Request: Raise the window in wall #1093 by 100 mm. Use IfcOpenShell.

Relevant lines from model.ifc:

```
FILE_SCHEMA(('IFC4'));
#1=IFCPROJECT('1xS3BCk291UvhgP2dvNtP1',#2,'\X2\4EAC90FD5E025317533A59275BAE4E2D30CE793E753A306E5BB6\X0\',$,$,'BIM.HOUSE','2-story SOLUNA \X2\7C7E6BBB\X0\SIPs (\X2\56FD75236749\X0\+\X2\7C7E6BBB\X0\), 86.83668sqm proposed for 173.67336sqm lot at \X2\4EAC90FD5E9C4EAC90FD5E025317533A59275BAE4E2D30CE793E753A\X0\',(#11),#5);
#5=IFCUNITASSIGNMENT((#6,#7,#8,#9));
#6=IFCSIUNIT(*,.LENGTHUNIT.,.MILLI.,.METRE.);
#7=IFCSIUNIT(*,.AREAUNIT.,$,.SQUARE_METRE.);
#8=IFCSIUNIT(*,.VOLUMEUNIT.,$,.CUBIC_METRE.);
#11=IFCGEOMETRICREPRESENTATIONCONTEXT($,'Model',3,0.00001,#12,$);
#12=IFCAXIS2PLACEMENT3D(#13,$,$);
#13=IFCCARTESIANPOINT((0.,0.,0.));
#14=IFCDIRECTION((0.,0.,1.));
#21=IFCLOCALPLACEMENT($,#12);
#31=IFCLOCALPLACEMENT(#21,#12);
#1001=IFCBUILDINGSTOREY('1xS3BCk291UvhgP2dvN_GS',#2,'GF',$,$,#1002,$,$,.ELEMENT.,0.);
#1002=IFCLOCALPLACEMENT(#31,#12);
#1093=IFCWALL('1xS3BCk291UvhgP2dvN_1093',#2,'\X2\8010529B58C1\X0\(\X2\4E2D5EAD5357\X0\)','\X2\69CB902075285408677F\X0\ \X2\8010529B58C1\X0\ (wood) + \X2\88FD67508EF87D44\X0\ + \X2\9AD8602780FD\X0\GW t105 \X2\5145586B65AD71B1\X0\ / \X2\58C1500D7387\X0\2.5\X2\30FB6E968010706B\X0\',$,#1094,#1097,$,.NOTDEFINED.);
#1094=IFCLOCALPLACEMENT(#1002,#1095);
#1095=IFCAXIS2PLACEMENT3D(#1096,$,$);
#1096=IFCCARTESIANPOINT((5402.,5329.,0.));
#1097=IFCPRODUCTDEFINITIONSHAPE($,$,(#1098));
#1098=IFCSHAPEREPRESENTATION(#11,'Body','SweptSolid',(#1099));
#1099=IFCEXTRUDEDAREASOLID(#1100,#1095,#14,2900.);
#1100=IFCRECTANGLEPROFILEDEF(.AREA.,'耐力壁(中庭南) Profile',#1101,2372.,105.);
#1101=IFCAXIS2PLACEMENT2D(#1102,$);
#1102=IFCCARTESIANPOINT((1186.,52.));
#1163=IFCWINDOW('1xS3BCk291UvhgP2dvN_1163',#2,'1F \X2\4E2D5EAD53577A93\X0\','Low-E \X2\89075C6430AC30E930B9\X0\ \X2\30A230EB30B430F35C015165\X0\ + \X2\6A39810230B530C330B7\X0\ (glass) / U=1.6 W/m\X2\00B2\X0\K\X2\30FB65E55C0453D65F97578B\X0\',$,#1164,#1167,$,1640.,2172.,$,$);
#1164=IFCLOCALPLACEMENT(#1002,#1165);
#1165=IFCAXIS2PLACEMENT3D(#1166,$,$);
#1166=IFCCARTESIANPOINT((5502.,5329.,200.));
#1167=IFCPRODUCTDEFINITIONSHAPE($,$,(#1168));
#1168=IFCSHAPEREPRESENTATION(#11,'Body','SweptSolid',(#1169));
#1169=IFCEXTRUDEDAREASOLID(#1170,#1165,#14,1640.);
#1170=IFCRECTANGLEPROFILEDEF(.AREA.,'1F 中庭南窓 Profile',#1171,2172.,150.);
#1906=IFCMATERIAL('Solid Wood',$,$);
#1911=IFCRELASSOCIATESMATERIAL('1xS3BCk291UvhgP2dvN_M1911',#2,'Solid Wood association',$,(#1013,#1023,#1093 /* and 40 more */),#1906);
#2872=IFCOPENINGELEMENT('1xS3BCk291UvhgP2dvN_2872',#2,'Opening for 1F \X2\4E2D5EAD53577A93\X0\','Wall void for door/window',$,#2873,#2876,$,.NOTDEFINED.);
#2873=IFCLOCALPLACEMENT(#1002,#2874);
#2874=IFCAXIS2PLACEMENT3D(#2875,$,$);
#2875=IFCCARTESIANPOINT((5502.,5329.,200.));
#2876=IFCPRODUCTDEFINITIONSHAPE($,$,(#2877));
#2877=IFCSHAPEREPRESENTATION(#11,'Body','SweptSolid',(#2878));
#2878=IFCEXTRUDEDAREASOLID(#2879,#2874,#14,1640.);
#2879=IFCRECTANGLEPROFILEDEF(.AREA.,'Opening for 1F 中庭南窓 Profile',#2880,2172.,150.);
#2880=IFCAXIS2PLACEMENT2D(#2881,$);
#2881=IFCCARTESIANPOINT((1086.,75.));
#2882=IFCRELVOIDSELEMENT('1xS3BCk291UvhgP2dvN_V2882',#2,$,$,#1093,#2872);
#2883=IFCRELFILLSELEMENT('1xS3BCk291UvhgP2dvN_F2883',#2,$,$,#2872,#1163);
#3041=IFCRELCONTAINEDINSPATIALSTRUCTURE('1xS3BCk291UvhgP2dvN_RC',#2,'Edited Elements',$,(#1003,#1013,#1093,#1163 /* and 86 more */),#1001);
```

```python
import numpy as np
import ifcopenshell
import ifcopenshell.api.geometry
import ifcopenshell.util.placement
import ifcopenshell.util.unit

model = ifcopenshell.open("model.ifc")
unit_scale = ifcopenshell.util.unit.calculate_unit_scale(model)

window = model.by_guid("1xS3BCk291UvhgP2dvN_1163")
opening = window.FillsVoids[0].RelatingOpeningElement
dz = 0.1 / unit_scale

shift = np.array([0.0, 0.0, dz])
# The window is not placed relative to its opening, so move both.
for product in (opening, window):
    matrix = ifcopenshell.util.placement.get_local_placement(product.ObjectPlacement)
    matrix[:3, 3] += shift
    ifcopenshell.api.geometry.edit_object_placement(model, product=product, matrix=matrix, is_si=False)

print(f"moved by {dz * unit_scale:+.3f} m")

model.write("model_rev.ifc")
```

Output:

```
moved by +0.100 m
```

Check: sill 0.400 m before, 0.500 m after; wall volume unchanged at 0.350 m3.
